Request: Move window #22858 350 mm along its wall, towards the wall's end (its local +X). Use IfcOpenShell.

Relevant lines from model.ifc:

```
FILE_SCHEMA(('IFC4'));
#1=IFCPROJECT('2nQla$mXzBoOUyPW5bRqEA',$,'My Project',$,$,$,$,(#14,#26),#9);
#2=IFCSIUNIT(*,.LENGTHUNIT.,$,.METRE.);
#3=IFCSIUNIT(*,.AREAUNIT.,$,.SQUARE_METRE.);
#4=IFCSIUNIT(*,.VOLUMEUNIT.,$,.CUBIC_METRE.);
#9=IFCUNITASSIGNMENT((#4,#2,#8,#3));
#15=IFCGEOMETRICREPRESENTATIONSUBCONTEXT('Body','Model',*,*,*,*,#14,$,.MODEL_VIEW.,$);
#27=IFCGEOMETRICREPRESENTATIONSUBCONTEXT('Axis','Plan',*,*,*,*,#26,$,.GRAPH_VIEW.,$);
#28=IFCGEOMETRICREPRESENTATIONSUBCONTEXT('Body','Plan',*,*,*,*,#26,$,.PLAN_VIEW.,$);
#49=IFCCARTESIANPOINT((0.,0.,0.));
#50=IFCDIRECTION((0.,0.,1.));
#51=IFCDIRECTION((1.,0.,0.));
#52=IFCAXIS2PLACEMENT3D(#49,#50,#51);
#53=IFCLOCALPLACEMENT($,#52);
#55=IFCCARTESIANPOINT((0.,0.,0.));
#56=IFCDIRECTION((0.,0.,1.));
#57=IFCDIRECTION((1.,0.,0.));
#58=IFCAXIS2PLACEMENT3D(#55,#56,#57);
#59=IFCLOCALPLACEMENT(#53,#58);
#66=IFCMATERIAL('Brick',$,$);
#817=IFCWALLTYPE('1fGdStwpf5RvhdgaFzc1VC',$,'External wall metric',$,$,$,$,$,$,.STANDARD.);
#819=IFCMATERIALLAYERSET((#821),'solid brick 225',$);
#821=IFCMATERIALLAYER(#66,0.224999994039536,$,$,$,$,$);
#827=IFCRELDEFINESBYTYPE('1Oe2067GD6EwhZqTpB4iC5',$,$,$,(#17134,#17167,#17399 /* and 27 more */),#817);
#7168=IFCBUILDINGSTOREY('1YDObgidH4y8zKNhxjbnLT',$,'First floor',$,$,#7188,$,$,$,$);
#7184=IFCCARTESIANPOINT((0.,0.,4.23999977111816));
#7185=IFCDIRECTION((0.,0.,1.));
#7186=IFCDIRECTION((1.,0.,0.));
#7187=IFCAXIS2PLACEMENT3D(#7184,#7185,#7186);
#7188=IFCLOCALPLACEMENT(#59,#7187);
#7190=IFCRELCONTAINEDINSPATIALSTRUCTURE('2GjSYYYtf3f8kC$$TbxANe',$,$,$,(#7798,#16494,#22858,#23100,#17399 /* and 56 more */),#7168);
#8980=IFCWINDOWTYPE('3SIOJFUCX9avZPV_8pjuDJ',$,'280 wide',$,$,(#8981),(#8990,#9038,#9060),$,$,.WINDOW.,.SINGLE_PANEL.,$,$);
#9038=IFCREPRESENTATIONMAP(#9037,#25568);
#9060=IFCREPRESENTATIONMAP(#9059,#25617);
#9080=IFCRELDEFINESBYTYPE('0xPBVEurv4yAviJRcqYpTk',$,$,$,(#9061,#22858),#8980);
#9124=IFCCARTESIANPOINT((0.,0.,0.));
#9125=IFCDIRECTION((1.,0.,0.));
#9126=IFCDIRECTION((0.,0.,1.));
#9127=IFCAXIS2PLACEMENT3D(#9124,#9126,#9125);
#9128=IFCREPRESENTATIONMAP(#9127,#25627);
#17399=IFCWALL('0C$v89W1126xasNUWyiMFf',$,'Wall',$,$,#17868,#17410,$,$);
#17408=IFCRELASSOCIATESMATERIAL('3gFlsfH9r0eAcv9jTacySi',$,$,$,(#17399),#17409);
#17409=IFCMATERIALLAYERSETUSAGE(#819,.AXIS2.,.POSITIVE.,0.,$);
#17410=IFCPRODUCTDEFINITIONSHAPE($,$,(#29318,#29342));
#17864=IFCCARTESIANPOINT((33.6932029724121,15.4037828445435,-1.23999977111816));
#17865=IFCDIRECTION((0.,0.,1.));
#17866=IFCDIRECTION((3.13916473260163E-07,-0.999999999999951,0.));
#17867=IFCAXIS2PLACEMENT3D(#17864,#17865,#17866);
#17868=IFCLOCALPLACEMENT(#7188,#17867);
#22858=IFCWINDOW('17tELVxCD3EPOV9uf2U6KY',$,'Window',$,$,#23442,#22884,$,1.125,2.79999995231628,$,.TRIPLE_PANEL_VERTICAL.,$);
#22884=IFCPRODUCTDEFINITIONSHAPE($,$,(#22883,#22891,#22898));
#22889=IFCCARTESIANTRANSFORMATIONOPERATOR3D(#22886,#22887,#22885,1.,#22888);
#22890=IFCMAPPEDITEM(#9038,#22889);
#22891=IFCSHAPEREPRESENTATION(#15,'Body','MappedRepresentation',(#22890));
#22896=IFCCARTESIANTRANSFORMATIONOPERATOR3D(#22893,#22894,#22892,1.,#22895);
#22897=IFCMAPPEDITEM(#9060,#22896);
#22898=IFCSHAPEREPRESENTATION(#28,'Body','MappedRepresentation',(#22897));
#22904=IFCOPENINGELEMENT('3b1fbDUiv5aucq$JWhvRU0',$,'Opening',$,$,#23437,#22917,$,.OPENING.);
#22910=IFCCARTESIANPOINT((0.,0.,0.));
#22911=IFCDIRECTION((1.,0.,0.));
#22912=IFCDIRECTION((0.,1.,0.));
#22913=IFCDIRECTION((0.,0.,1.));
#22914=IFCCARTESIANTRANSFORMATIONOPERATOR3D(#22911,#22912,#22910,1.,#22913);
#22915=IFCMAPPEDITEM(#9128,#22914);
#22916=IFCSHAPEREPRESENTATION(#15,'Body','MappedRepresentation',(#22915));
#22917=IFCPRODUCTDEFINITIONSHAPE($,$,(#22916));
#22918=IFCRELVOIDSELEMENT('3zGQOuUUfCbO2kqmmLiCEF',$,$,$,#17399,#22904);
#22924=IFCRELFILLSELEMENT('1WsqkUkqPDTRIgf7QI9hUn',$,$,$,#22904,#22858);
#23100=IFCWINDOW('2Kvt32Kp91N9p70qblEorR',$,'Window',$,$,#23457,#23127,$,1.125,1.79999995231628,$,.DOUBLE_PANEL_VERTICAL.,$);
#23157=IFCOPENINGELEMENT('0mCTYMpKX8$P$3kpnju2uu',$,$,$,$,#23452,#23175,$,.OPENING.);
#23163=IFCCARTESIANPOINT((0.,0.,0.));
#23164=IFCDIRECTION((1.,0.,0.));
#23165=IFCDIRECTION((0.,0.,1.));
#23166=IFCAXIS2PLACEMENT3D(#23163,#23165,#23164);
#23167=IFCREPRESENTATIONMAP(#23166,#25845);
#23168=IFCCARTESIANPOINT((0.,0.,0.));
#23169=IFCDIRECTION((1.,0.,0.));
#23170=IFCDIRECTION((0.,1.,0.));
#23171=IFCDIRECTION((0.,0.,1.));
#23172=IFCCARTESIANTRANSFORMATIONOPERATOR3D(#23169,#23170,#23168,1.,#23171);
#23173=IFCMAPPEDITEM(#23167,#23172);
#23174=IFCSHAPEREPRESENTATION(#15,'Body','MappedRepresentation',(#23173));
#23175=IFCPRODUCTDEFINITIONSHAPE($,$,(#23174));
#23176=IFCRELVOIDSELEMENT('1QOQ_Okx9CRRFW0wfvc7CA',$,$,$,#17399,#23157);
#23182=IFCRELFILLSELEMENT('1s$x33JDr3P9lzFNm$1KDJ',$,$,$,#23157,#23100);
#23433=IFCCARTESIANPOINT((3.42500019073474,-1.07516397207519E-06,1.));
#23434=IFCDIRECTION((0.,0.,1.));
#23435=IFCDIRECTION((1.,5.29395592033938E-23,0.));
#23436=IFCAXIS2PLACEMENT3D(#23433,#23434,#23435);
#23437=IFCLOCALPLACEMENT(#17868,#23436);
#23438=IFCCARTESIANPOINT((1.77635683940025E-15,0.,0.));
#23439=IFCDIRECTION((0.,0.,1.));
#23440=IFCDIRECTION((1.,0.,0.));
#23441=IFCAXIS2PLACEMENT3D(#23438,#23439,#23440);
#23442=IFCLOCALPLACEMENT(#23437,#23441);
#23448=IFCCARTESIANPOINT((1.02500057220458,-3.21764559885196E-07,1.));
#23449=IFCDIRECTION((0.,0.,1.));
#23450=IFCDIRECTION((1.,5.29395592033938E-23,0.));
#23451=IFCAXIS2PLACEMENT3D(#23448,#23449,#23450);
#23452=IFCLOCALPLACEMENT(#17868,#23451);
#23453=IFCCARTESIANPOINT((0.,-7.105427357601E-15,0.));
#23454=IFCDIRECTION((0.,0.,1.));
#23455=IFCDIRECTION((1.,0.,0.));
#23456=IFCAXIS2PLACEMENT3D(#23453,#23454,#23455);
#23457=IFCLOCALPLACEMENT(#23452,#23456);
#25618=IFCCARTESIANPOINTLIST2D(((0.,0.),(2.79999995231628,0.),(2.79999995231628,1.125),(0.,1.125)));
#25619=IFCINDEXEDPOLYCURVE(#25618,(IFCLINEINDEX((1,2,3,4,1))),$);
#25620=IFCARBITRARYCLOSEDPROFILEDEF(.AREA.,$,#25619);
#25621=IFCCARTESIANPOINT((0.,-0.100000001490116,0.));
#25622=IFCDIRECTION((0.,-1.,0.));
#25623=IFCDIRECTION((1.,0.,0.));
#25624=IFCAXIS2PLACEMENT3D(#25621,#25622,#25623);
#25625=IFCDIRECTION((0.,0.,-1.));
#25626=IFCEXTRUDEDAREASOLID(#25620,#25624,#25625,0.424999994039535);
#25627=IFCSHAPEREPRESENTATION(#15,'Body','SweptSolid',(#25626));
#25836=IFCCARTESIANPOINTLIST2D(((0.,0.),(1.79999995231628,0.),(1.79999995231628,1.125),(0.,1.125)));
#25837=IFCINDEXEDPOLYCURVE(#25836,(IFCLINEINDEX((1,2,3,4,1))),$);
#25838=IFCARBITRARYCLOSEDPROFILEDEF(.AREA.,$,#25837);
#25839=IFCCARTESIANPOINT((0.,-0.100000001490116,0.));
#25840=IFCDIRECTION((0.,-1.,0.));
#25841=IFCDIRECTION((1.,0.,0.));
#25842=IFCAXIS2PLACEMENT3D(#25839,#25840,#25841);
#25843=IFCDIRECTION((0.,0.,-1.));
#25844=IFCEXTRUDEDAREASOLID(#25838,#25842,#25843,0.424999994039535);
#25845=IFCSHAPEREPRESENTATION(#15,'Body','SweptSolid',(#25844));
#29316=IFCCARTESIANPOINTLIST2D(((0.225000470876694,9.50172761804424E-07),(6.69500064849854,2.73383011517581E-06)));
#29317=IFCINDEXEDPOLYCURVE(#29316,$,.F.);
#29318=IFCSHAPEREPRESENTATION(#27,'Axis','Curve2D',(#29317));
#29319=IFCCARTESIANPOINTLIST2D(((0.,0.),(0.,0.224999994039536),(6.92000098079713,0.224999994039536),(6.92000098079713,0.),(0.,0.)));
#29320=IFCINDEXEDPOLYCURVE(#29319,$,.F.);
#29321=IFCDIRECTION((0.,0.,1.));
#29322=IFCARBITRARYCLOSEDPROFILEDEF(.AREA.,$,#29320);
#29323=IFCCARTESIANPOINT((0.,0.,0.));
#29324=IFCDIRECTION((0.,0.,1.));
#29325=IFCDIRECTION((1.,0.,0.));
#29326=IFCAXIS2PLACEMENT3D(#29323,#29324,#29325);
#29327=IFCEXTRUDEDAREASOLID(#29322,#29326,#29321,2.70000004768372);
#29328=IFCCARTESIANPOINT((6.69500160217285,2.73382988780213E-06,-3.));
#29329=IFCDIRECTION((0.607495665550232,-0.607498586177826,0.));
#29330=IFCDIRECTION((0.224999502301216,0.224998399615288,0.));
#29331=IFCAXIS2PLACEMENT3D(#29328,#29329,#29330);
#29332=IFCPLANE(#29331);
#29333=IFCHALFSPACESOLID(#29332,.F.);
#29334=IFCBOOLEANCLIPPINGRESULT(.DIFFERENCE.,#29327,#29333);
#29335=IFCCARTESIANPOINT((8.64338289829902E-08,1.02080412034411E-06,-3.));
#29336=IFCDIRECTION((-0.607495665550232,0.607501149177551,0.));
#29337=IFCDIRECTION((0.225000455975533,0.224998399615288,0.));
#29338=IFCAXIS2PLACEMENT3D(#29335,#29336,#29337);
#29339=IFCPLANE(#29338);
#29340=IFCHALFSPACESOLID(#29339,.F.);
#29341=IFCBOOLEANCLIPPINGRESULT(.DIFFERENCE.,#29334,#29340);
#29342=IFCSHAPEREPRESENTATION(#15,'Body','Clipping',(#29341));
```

```python
import ifcopenshell
import ifcopenshell.api.geometry
import ifcopenshell.util.placement
import ifcopenshell.util.unit

model = ifcopenshell.open("model.ifc")
unit_scale = ifcopenshell.util.unit.calculate_unit_scale(model)

window = model.by_guid("17tELVxCD3EPOV9uf2U6KY")
opening = window.FillsVoids[0].RelatingOpeningElement
wall = opening.VoidsElements[0].RelatingBuildingElement

wall_matrix = ifcopenshell.util.placement.get_local_placement(wall.ObjectPlacement)
shift = wall_matrix[:3, 0] * 0.35 / unit_scale
before = ifcopenshell.util.placement.get_local_placement(window.ObjectPlacement)[:3, 3].copy()

# The window is placed relative to its opening, so it follows when the opening moves.
matrix = ifcopenshell.util.placement.get_local_placement(opening.ObjectPlacement)
matrix[:3, 3] += shift
ifcopenshell.api.geometry.edit_object_placement(
    model, product=opening, matrix=matrix, is_si=False, should_transform_children=True
)

after = ifcopenshell.util.placement.get_local_placement(window.ObjectPlacement)[:3, 3]
print("window moved by", (after - before).round(3) + 0.0)

model.write("model_v2.ifc")
```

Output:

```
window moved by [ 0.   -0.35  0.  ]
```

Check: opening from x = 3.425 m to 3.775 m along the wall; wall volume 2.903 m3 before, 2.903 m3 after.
